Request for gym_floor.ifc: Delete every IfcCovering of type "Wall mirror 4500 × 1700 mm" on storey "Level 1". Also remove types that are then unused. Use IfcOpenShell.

First a look at what the model holds.

```python
import ifcopenshell
import ifcopenshell.util.element

model = ifcopenshell.open("gym_floor.ifc")
print(model.schema)
storey = next(s for s in model.by_type("IfcBuildingStorey") if s.Name == "Level 1")
coverings = [e for e in ifcopenshell.util.element.get_decomposition(storey) if e.is_a("IfcCovering")]
seen = {}
for e in coverings:
    element_type = ifcopenshell.util.element.get_type(e)
    name = element_type.Name if element_type not in (None, e) else None
    seen[name] = seen.get(name, 0) + 1
for name, count in sorted(seen.items(), key=str):
    print(count, "x", name)
```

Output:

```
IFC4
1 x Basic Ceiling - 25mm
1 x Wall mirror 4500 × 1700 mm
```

```python
import ifcopenshell
import ifcopenshell.api.root
import ifcopenshell.util.element

model = ifcopenshell.open("gym_floor.ifc")

storey = next(s for s in model.by_type("IfcBuildingStorey") if s.Name == "Level 1")
coverings = [e for e in ifcopenshell.util.element.get_decomposition(storey) if e.is_a("IfcCovering")]
targets = [e for e in coverings if (t := ifcopenshell.util.element.get_type(e)) not in (None, e) and t.Name == "Wall mirror 4500 × 1700 mm"]
types = {ifcopenshell.util.element.get_type(e) for e in targets} - {None, *targets}

for e in targets:
    ifcopenshell.api.root.remove_product(model, product=e)
print(len(targets), "removed")

unused = [t for t in types if not ifcopenshell.util.element.get_types(t)]
for t in unused:
    ifcopenshell.api.root.remove_product(model, product=t)
print(len(unused), "unused types removed")

model.write("gym_floor_edited.ifc")
```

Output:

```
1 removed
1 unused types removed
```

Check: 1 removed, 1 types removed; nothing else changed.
